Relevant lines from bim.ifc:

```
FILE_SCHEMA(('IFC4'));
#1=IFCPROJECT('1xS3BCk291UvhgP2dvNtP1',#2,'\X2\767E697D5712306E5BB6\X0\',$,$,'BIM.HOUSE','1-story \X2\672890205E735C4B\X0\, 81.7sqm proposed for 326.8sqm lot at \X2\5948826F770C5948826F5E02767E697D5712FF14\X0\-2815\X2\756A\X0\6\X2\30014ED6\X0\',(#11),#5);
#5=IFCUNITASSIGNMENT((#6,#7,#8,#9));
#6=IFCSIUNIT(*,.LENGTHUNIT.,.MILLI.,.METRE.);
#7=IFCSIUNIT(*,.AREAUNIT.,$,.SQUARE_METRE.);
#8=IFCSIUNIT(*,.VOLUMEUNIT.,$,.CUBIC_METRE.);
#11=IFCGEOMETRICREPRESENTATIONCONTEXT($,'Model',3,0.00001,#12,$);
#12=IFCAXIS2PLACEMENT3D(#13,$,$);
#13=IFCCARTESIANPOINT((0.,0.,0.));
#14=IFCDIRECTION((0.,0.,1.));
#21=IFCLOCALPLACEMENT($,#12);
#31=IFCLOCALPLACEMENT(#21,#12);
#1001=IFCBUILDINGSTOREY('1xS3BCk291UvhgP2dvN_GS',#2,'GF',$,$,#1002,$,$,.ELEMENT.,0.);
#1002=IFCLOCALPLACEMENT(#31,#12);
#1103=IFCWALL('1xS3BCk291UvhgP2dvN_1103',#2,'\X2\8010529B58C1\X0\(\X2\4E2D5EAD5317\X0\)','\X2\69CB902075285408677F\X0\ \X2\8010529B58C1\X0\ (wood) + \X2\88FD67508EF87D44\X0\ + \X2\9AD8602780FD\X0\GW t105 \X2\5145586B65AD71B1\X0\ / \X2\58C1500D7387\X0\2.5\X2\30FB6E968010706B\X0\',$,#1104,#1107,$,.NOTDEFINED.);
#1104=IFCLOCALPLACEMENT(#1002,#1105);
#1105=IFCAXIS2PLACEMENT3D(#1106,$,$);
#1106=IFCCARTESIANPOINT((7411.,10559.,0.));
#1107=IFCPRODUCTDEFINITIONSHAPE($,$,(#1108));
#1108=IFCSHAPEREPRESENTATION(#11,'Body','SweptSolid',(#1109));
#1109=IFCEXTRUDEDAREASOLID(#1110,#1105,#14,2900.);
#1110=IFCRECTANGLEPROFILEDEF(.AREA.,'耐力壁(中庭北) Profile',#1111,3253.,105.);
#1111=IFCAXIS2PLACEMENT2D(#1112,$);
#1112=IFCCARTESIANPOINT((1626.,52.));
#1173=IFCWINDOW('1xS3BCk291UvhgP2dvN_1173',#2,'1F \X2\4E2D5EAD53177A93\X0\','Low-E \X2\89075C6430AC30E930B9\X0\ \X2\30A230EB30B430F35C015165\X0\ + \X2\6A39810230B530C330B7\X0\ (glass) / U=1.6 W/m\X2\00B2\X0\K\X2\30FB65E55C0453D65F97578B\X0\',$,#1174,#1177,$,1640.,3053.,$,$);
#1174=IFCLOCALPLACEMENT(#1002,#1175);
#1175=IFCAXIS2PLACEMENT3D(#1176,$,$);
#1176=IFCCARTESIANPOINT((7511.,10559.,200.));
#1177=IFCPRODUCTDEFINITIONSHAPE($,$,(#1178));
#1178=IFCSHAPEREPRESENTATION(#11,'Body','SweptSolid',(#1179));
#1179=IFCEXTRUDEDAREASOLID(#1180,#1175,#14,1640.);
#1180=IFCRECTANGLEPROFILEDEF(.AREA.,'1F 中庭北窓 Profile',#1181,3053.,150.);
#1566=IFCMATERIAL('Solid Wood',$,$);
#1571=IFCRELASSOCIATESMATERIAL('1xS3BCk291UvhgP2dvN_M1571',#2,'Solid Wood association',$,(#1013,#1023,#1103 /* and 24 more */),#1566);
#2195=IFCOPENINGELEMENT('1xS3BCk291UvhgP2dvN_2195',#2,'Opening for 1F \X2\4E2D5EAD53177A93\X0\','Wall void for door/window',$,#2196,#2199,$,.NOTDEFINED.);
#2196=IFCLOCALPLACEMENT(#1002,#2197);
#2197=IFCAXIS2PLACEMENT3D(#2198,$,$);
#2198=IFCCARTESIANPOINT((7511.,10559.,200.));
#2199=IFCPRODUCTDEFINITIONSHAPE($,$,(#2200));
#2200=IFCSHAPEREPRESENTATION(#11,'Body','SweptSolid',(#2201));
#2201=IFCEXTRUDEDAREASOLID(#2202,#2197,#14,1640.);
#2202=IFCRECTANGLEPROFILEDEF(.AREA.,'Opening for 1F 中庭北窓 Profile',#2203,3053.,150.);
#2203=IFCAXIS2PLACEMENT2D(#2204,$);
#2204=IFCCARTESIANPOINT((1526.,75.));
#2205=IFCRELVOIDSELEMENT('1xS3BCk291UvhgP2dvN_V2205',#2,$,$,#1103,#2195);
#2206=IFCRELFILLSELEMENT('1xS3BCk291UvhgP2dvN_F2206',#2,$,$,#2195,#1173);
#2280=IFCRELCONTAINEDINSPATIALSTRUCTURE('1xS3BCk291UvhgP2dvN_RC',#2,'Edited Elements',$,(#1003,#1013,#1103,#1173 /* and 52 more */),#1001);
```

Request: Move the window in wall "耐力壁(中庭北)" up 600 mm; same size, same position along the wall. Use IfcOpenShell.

```python
import numpy as np
import ifcopenshell
import ifcopenshell.api.geometry
import ifcopenshell.util.placement
import ifcopenshell.util.unit

model = ifcopenshell.open("bim.ifc")
unit_scale = ifcopenshell.util.unit.calculate_unit_scale(model)

window = model.by_guid("1xS3BCk291UvhgP2dvN_1173")
opening = window.FillsVoids[0].RelatingOpeningElement
dz = 0.6 / unit_scale

shift = np.array([0.0, 0.0, dz])
# The window is not placed relative to its opening, so move both.
for product in (opening, window):
    matrix = ifcopenshell.util.placement.get_local_placement(product.ObjectPlacement)
    matrix[:3, 3] += shift
    ifcopenshell.api.geometry.edit_object_placement(model, product=product, matrix=matrix, is_si=False)

print(f"moved by {dz * unit_scale:+.3f} m")

model.write("bim_edited.ifc")
```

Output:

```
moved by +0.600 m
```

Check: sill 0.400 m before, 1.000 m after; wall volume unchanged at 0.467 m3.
